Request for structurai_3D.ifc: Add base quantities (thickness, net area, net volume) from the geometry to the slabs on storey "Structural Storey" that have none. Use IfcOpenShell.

First a look at what the model holds.

```python
import ifcopenshell
import ifcopenshell.util.element
import ifcopenshell.util.unit

model = ifcopenshell.open("structurai_3D.ifc")
print(model.schema)
for unit_type in ("LENGTHUNIT", "AREAUNIT", "VOLUMEUNIT"):
    print(unit_type, ifcopenshell.util.unit.calculate_unit_scale(model, unit_type))
storey = next(s for s in model.by_type("IfcBuildingStorey") if s.Name == "Structural Storey")
slabs = [e for e in ifcopenshell.util.element.get_decomposition(storey) if e.is_a("IfcSlab")]
for e in sorted(slabs, key=lambda e: e.id()):
    print(e.id(), e.is_a(), e.Name, list(ifcopenshell.util.element.get_psets(e, qtos_only=True)), sep=" | ")
```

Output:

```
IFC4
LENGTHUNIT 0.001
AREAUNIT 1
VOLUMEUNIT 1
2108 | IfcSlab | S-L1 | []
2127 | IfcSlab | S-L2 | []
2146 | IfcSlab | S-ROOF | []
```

```python
import ifcopenshell
import ifcopenshell.api.pset
import ifcopenshell.geom
import ifcopenshell.util.element
import ifcopenshell.util.shape
import ifcopenshell.util.unit

model = ifcopenshell.open("structurai_3D.ifc")
unit_scale = ifcopenshell.util.unit.calculate_unit_scale(model)
area_scale = ifcopenshell.util.unit.calculate_unit_scale(model, "AREAUNIT")
volume_scale = ifcopenshell.util.unit.calculate_unit_scale(model, "VOLUMEUNIT")
settings = ifcopenshell.geom.settings()

storey = next(s for s in model.by_type("IfcBuildingStorey") if s.Name == "Structural Storey")
slabs = [e for e in ifcopenshell.util.element.get_decomposition(storey) if e.is_a("IfcSlab")]

for e in sorted(slabs, key=lambda e: e.id()):
    if ifcopenshell.util.element.get_psets(e, qtos_only=True, should_inherit=False):
        continue
    # Geometry comes back in metres, in the element's own axes.
    shape = ifcopenshell.geom.create_shape(settings, e)
    values = {
        "Width": ifcopenshell.util.shape.get_z(shape.geometry) / unit_scale,
        "NetArea": ifcopenshell.util.shape.get_footprint_area(shape.geometry) / area_scale,
        "NetVolume": ifcopenshell.util.shape.get_volume(shape.geometry) / volume_scale,
    }
    qto = ifcopenshell.api.pset.add_qto(model, product=e, name="Qto_SlabBaseQuantities")
    ifcopenshell.api.pset.edit_qto(model, qto=qto, properties=values)
    print(e.id(), {k: round(v, 3) for k, v in values.items()})

model.write("structurai_3D-out.ifc")
```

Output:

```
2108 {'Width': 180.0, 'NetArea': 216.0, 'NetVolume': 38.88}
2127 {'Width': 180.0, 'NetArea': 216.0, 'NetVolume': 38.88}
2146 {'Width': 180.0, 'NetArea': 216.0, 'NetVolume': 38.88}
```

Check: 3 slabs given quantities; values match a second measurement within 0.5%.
